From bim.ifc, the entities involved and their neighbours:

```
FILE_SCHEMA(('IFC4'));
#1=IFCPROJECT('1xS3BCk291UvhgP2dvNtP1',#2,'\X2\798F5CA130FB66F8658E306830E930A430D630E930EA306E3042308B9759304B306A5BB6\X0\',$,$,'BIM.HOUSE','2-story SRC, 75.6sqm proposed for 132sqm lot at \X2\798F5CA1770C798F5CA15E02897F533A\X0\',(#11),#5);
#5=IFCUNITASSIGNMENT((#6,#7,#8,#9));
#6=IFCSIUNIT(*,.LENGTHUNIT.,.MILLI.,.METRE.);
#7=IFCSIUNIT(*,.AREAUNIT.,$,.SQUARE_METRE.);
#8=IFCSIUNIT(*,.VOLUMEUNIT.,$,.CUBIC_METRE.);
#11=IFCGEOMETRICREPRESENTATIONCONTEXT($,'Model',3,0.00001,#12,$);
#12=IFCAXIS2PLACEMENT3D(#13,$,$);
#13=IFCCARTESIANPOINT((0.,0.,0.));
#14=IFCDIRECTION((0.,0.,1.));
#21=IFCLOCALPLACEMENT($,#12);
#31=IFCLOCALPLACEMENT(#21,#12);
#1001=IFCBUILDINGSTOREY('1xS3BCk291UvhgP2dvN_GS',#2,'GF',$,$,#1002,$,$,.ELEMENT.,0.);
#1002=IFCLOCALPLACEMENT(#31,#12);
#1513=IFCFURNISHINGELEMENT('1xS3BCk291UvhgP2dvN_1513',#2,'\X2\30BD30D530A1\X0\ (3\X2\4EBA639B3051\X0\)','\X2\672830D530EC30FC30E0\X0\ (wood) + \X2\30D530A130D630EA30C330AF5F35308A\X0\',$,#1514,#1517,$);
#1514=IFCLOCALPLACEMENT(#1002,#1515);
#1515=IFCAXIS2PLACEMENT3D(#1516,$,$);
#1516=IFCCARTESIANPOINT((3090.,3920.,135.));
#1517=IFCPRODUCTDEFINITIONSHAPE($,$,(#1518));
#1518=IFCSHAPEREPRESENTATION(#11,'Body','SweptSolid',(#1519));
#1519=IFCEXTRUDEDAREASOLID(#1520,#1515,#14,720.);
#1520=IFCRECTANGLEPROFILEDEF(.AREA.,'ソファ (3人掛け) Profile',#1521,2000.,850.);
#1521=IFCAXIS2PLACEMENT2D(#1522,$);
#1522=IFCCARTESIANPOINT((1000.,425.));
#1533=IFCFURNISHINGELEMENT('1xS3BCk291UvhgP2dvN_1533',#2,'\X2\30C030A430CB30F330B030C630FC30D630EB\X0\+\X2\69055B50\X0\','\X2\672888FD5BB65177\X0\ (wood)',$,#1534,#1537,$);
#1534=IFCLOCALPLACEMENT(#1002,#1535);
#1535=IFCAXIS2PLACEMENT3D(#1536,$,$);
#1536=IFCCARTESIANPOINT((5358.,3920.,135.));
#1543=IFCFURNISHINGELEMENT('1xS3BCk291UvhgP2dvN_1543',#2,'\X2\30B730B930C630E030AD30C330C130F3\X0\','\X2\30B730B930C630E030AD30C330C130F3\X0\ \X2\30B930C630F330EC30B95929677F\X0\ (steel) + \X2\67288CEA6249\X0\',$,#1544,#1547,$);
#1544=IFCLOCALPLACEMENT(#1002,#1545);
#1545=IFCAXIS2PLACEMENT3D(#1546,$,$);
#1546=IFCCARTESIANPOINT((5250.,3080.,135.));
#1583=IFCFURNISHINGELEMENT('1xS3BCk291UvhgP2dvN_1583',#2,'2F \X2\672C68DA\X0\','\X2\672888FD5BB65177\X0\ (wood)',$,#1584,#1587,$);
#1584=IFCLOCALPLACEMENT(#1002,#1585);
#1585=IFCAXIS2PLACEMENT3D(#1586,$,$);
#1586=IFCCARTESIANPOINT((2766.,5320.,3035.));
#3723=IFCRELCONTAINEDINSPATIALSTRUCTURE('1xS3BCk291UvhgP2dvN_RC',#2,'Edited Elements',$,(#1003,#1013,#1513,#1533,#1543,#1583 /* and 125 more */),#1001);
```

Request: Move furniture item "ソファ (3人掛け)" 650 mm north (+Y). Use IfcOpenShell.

```python
import ifcopenshell
import ifcopenshell.api.geometry
import ifcopenshell.util.placement
import ifcopenshell.util.unit

model = ifcopenshell.open("bim.ifc")
unit_scale = ifcopenshell.util.unit.calculate_unit_scale(model)

item = model.by_guid("1xS3BCk291UvhgP2dvN_1513")
matrix = ifcopenshell.util.placement.get_local_placement(item.ObjectPlacement)
matrix[1, 3] += 0.65 / unit_scale
ifcopenshell.api.geometry.edit_object_placement(model, product=item, matrix=matrix, is_si=False)

print(ifcopenshell.util.placement.get_local_placement(item.ObjectPlacement).round(3) + 0.0)

model.write("bim_rev.ifc")
```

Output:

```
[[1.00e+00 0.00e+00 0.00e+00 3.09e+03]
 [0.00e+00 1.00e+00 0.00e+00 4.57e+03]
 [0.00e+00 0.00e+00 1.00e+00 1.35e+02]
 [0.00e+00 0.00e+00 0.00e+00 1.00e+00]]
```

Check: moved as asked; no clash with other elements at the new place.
